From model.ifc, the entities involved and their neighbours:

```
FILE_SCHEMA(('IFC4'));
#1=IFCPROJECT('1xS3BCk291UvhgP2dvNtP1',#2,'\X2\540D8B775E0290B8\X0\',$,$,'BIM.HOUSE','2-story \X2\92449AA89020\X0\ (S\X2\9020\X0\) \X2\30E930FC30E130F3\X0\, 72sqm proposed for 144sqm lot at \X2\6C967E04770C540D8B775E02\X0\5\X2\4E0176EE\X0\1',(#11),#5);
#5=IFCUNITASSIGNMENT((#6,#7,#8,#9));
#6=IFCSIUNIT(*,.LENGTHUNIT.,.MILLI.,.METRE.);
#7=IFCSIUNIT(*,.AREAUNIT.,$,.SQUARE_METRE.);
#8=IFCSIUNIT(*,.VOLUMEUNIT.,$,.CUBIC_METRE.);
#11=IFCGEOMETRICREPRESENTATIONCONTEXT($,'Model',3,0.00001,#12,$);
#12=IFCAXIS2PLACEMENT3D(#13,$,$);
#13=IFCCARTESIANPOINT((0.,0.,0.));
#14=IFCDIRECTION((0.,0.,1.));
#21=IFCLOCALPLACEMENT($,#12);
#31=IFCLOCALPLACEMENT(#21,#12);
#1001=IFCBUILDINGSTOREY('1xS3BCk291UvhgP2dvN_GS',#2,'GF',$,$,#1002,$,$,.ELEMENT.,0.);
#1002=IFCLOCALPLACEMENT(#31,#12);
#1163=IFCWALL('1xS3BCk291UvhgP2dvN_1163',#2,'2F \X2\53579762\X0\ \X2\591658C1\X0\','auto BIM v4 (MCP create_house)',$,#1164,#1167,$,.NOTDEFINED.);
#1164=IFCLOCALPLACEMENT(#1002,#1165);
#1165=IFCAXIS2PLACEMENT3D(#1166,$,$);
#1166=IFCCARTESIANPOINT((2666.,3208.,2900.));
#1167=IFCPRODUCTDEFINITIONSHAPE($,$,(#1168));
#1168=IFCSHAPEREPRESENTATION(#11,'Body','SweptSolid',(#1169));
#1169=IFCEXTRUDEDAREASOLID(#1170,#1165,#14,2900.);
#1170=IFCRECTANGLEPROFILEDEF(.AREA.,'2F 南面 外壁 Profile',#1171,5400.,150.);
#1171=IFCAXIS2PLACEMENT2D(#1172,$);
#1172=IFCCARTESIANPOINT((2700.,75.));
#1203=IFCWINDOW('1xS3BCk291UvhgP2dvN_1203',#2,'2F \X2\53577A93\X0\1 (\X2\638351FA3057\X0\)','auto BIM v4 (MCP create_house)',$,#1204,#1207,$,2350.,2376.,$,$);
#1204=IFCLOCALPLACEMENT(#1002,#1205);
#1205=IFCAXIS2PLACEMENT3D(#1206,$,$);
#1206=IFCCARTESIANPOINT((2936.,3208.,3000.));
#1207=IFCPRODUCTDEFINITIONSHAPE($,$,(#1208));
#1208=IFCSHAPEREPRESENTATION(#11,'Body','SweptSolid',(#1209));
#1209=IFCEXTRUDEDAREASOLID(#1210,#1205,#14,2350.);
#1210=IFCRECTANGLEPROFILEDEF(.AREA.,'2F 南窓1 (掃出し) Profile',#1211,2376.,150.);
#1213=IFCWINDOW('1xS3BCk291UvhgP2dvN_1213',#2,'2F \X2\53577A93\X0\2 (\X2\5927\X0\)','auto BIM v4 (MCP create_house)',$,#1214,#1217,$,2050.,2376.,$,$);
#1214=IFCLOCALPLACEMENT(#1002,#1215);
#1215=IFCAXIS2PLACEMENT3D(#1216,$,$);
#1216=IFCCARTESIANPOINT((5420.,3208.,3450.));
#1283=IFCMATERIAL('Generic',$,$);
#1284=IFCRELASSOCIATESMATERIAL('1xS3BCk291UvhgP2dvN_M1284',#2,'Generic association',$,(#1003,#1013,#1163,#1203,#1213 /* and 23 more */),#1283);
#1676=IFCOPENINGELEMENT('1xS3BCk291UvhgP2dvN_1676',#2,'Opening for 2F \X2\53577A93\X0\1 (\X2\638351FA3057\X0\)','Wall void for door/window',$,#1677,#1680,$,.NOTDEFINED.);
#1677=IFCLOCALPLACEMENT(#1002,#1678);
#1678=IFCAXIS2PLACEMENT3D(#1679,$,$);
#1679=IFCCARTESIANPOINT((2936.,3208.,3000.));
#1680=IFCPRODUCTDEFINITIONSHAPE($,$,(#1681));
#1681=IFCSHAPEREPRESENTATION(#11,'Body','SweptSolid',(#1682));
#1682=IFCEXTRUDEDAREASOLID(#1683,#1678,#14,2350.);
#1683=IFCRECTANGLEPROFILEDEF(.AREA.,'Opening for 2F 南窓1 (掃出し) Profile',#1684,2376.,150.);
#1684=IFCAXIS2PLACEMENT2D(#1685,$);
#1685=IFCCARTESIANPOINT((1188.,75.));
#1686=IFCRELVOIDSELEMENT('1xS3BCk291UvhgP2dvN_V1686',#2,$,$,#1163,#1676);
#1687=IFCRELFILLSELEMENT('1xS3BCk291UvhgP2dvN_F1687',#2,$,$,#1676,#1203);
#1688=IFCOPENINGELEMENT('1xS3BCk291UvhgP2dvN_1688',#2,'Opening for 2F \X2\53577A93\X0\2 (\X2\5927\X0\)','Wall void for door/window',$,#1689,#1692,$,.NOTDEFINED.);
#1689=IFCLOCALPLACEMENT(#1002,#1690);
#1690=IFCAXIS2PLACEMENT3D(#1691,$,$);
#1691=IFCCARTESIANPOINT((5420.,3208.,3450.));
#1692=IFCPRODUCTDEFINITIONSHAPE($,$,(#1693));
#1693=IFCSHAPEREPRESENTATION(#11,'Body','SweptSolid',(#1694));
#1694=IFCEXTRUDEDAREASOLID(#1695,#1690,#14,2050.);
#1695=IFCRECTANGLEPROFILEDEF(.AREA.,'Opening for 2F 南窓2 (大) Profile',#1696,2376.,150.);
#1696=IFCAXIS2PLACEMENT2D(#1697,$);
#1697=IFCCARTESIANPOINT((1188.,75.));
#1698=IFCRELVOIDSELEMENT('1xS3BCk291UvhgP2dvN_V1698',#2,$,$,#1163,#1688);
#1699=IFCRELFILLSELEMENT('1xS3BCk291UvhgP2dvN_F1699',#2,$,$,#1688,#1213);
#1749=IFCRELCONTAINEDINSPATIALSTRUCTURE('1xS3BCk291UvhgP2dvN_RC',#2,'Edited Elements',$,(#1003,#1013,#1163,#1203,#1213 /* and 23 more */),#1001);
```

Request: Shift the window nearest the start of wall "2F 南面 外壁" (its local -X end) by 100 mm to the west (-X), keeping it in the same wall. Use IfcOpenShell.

```python
import ifcopenshell
import ifcopenshell.api.geometry
import ifcopenshell.util.placement
import ifcopenshell.util.unit

model = ifcopenshell.open("model.ifc")
unit_scale = ifcopenshell.util.unit.calculate_unit_scale(model)

window = model.by_id(1203)
opening = window.FillsVoids[0].RelatingOpeningElement
wall = opening.VoidsElements[0].RelatingBuildingElement

wall_matrix = ifcopenshell.util.placement.get_local_placement(wall.ObjectPlacement)
shift = wall_matrix[:3, 0] * -0.1 / unit_scale
before = ifcopenshell.util.placement.get_local_placement(window.ObjectPlacement)[:3, 3].copy()

# The window is not placed relative to its opening, so move both.
for product in (opening, window):
    matrix = ifcopenshell.util.placement.get_local_placement(product.ObjectPlacement)
    matrix[:3, 3] += shift
    ifcopenshell.api.geometry.edit_object_placement(model, product=product, matrix=matrix, is_si=False)

after = ifcopenshell.util.placement.get_local_placement(window.ObjectPlacement)[:3, 3]
print("window moved by", (after - before).round(3) + 0.0)

model.write("model_edited.ifc")
```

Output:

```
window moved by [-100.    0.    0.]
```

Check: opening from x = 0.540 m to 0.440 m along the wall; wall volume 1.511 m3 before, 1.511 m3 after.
